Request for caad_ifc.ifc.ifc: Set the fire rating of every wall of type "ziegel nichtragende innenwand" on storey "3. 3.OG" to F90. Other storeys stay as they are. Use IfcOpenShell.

First a look at what the model holds.

```python
import ifcopenshell
import ifcopenshell.util.element

model = ifcopenshell.open("caad_ifc.ifc.ifc")
print(model.schema)
storey = next(s for s in model.by_type("IfcBuildingStorey") if s.Name == "3. 3.OG")
walls = [e for e in ifcopenshell.util.element.get_decomposition(storey) if e.is_a("IfcWall")]
seen = {}
for e in walls:
    element_type = ifcopenshell.util.element.get_type(e)
    key = (element_type.Name if element_type != e and element_type else None, ifcopenshell.util.element.get_pset(e, "Pset_WallCommon", "FireRating"))
    seen[key] = seen.get(key, 0) + 1
for (name, value), count in sorted(seen.items(), key=str):
    print(count, "x", name, "|", value)
```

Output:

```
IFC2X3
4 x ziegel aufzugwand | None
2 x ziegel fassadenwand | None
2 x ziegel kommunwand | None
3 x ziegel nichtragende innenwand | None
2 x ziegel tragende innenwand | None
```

```python
import ifcopenshell
import ifcopenshell.api.pset
import ifcopenshell.util.element

model = ifcopenshell.open("caad_ifc.ifc.ifc")

storey = next(s for s in model.by_type("IfcBuildingStorey") if s.Name == "3. 3.OG")
walls = [e for e in ifcopenshell.util.element.get_decomposition(storey) if e.is_a("IfcWall")]

count = 0
for e in walls:
    element_type = ifcopenshell.util.element.get_type(e)
    if element_type in (None, e) or element_type.Name != "ziegel nichtragende innenwand":
        continue
    # add_pset returns the element's existing set when there is one.
    pset = ifcopenshell.api.pset.add_pset(model, product=e, name="Pset_WallCommon")
    ifcopenshell.api.pset.edit_pset(model, pset=pset, properties={"FireRating": "F90"})
    count += 1

print(count, "walls updated")

model.write("caad_ifc.ifc-out.ifc")
```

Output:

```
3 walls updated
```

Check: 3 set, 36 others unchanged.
